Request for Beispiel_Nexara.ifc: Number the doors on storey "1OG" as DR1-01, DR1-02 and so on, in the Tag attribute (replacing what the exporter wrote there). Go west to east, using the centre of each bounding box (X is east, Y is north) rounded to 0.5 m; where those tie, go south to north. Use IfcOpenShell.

First a look at what the model holds.

```python
import ifcopenshell
import ifcopenshell.util.element
import ifcopenshell.util.placement

model = ifcopenshell.open("Beispiel_Nexara.ifc")
print(model.schema)
storey = next(s for s in model.by_type("IfcBuildingStorey") if s.Name == "1OG")
doors = [e for e in ifcopenshell.util.element.get_decomposition(storey) if e.is_a("IfcDoor")]
for e in sorted(doors, key=lambda e: e.id()):
    origin = ifcopenshell.util.placement.get_local_placement(e.ObjectPlacement)[:3, 3]
    print(e.id(), e.Tag, e.Name, origin.round(2) + 0.0, sep=" | ")
```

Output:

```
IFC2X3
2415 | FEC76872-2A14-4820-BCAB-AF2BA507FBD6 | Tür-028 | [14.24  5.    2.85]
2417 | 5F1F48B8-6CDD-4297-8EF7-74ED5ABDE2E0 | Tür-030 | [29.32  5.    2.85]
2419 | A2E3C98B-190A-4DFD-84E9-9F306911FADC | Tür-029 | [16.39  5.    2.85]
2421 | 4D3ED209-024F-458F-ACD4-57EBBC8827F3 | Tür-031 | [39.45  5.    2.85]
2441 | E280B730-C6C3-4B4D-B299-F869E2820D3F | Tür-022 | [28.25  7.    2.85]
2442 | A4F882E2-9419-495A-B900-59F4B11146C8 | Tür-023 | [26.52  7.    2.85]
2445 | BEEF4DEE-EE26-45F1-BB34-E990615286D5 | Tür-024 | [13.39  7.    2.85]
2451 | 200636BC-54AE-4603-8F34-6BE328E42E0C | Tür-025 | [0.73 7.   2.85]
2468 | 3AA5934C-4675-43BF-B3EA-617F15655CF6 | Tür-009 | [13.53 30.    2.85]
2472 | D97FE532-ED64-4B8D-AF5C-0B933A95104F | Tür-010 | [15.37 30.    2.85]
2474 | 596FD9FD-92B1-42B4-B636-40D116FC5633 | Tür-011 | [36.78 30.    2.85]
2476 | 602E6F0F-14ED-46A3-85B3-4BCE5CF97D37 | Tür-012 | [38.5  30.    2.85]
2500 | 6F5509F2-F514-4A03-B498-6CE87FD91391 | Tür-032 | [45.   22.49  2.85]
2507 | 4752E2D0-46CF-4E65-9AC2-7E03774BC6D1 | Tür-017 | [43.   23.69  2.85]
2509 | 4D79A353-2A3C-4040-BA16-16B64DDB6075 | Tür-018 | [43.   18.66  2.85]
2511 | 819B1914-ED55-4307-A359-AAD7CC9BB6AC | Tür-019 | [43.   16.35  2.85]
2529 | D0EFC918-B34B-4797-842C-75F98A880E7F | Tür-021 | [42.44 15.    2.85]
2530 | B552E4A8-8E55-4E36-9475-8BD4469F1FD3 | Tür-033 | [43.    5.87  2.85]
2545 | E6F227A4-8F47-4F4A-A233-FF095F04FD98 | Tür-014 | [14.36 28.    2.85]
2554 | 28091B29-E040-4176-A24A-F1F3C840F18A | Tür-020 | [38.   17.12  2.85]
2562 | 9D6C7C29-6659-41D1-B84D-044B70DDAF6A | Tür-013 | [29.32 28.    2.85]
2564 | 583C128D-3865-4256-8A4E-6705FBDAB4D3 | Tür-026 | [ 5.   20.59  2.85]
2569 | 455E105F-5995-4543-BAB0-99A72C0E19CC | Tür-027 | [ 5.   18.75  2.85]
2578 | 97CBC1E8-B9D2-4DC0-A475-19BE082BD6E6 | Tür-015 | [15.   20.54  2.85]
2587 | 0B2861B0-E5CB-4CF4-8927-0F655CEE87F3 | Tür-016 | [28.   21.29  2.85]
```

```python
import ifcopenshell
import ifcopenshell.geom
import ifcopenshell.util.element
import ifcopenshell.util.shape

model = ifcopenshell.open("Beispiel_Nexara.ifc")
settings = ifcopenshell.geom.settings()
settings.set("use-world-coords", True)


def centre(element):
    shape = ifcopenshell.geom.create_shape(settings, element)
    return ifcopenshell.util.shape.get_bbox_centroid(shape.geometry)


storey = next(s for s in model.by_type("IfcBuildingStorey") if s.Name == "1OG")
doors = [e for e in ifcopenshell.util.element.get_decomposition(storey) if e.is_a("IfcDoor")]

# Insertion points can sit at a corner or the storey origin, so sort by the geometry (in metres).
centres = {e: centre(e) for e in doors}
doors.sort(key=lambda e: (round(centres[e][0] / 0.5), centres[e][1]))

for i, e in enumerate(doors, start=1):
    number = f"DR1-{i:02d}"
    e.Tag = number
    print(e.id(), number)

model.write("Beispiel_Nexara_updated.ifc")
```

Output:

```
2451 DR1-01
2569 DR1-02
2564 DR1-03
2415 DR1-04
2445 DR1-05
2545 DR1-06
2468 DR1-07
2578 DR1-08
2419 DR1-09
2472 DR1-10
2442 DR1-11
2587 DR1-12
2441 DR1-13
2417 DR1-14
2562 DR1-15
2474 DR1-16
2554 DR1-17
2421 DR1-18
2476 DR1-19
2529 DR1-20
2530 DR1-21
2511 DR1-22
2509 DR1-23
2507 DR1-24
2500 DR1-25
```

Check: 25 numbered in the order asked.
